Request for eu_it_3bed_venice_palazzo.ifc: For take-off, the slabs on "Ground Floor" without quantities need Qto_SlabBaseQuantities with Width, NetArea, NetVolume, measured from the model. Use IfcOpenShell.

First a look at what the model holds.

```python
import ifcopenshell
import ifcopenshell.util.element
import ifcopenshell.util.unit

model = ifcopenshell.open("eu_it_3bed_venice_palazzo.ifc")
print(model.schema)
for unit_type in ("LENGTHUNIT", "AREAUNIT", "VOLUMEUNIT"):
    print(unit_type, ifcopenshell.util.unit.calculate_unit_scale(model, unit_type))
storey = next(s for s in model.by_type("IfcBuildingStorey") if s.Name == "Ground Floor")
slabs = [e for e in ifcopenshell.util.element.get_decomposition(storey) if e.is_a("IfcSlab")]
for e in sorted(slabs, key=lambda e: e.id()):
    print(e.id(), e.is_a(), e.Name, list(ifcopenshell.util.element.get_psets(e, qtos_only=True)), sep=" | ")
```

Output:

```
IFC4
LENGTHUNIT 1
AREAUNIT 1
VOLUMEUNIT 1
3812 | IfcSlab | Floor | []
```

```python
import ifcopenshell
import ifcopenshell.api.pset
import ifcopenshell.geom
import ifcopenshell.util.element
import ifcopenshell.util.shape
import ifcopenshell.util.unit

model = ifcopenshell.open("eu_it_3bed_venice_palazzo.ifc")
unit_scale = ifcopenshell.util.unit.calculate_unit_scale(model)
area_scale = ifcopenshell.util.unit.calculate_unit_scale(model, "AREAUNIT")
volume_scale = ifcopenshell.util.unit.calculate_unit_scale(model, "VOLUMEUNIT")
settings = ifcopenshell.geom.settings()

storey = next(s for s in model.by_type("IfcBuildingStorey") if s.Name == "Ground Floor")
slabs = [e for e in ifcopenshell.util.element.get_decomposition(storey) if e.is_a("IfcSlab")]

for e in sorted(slabs, key=lambda e: e.id()):
    if ifcopenshell.util.element.get_psets(e, qtos_only=True, should_inherit=False):
        continue
    # Geometry comes back in metres, in the element's own axes.
    shape = ifcopenshell.geom.create_shape(settings, e)
    values = {
        "Width": ifcopenshell.util.shape.get_z(shape.geometry) / unit_scale,
        "NetArea": ifcopenshell.util.shape.get_footprint_area(shape.geometry) / area_scale,
        "NetVolume": ifcopenshell.util.shape.get_volume(shape.geometry) / volume_scale,
    }
    qto = ifcopenshell.api.pset.add_qto(model, product=e, name="Qto_SlabBaseQuantities")
    ifcopenshell.api.pset.edit_qto(model, qto=qto, properties=values)
    print(e.id(), {k: round(v, 3) for k, v in values.items()})

model.write("eu_it_3bed_venice_palazzo_updated.ifc")
```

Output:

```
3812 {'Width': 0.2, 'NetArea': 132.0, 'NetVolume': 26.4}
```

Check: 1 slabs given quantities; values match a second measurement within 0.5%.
